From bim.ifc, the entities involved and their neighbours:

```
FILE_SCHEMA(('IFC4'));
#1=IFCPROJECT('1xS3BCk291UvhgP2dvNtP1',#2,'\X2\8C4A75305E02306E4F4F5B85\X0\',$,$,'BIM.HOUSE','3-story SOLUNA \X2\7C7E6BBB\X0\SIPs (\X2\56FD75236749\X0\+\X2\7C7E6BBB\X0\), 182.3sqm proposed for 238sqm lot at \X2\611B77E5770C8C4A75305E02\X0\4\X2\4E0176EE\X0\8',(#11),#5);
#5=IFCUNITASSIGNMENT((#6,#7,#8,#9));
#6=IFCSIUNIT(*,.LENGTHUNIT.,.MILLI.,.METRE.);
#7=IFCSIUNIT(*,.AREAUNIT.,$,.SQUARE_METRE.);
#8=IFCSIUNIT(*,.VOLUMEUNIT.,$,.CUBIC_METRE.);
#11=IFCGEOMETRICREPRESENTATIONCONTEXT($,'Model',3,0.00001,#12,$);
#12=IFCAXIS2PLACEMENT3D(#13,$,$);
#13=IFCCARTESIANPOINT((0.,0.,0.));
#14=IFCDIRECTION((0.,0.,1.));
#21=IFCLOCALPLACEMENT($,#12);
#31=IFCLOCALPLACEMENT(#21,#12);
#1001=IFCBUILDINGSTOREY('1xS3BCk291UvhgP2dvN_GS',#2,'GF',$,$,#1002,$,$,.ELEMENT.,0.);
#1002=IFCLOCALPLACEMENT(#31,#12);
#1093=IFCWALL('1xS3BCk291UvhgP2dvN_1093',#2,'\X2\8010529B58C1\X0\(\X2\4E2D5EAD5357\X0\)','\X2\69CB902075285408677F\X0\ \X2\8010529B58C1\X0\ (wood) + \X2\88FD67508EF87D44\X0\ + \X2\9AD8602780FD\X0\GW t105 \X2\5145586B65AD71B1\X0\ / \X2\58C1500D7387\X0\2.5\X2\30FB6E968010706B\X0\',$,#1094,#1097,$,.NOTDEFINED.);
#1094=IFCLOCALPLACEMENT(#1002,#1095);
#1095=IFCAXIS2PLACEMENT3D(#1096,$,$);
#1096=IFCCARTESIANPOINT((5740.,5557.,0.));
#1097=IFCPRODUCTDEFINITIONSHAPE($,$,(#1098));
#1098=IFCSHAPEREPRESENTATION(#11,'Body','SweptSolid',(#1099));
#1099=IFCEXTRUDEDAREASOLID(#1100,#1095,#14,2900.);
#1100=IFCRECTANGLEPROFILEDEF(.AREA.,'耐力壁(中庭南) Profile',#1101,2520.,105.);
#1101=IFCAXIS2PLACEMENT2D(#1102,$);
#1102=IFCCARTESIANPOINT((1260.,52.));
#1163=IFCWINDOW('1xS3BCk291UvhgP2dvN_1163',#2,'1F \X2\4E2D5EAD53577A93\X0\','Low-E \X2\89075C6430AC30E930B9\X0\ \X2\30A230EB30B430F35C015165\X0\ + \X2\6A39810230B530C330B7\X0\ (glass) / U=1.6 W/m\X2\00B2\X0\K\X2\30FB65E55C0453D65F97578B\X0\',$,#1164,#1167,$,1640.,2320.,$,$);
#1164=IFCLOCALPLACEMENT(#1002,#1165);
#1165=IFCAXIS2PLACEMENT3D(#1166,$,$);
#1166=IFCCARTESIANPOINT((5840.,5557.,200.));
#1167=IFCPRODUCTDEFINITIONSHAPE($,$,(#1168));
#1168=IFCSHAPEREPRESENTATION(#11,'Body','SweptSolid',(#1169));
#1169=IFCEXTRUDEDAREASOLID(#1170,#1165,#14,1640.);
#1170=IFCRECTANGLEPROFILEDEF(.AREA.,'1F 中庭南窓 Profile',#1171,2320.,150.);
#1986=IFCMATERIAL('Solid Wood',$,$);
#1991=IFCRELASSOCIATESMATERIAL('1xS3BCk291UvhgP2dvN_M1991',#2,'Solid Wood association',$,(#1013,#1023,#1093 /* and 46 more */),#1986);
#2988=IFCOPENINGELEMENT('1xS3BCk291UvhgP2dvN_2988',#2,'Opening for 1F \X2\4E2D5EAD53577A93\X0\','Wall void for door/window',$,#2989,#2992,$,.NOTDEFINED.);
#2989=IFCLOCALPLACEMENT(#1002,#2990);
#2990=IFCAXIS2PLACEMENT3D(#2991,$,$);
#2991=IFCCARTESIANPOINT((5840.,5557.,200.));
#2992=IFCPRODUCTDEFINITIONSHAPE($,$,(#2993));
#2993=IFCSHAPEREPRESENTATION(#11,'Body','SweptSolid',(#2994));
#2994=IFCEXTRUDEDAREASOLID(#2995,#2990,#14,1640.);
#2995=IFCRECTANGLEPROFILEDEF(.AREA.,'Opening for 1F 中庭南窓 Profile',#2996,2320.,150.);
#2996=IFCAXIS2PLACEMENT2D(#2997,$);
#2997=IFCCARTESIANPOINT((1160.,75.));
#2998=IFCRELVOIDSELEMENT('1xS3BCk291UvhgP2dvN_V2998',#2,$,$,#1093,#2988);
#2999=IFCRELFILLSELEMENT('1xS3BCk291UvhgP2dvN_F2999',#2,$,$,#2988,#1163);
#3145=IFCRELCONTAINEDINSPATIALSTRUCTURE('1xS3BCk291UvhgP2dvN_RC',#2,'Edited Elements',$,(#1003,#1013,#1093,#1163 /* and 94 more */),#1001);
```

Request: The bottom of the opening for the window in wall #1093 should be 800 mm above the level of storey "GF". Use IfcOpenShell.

```python
import numpy as np
import ifcopenshell
import ifcopenshell.api.geometry
import ifcopenshell.geom
import ifcopenshell.util.element
import ifcopenshell.util.placement
import ifcopenshell.util.shape
import ifcopenshell.util.unit

model = ifcopenshell.open("bim.ifc")
unit_scale = ifcopenshell.util.unit.calculate_unit_scale(model)

window = model.by_guid("1xS3BCk291UvhgP2dvN_1163")
opening = window.FillsVoids[0].RelatingOpeningElement
storey = ifcopenshell.util.element.get_container(window, ifc_class="IfcBuildingStorey")
level = ifcopenshell.util.placement.get_local_placement(storey.ObjectPlacement)[2, 3]

# The opening's origin need not be at the sill, so measure its lowest point.
shape = ifcopenshell.geom.create_shape(ifcopenshell.geom.settings(), opening)
bottom = ifcopenshell.util.shape.get_shape_bottom_elevation(shape, shape.geometry) / unit_scale
dz = level + 800.0 - bottom

shift = np.array([0.0, 0.0, dz])
# The window is not placed relative to its opening, so move both.
for product in (opening, window):
    matrix = ifcopenshell.util.placement.get_local_placement(product.ObjectPlacement)
    matrix[:3, 3] += shift
    ifcopenshell.api.geometry.edit_object_placement(model, product=product, matrix=matrix, is_si=False)

print(f"moved by {dz * unit_scale:+.3f} m")

model.write("bim_rev.ifc")
```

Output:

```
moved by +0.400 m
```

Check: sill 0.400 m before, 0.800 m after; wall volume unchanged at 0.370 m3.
